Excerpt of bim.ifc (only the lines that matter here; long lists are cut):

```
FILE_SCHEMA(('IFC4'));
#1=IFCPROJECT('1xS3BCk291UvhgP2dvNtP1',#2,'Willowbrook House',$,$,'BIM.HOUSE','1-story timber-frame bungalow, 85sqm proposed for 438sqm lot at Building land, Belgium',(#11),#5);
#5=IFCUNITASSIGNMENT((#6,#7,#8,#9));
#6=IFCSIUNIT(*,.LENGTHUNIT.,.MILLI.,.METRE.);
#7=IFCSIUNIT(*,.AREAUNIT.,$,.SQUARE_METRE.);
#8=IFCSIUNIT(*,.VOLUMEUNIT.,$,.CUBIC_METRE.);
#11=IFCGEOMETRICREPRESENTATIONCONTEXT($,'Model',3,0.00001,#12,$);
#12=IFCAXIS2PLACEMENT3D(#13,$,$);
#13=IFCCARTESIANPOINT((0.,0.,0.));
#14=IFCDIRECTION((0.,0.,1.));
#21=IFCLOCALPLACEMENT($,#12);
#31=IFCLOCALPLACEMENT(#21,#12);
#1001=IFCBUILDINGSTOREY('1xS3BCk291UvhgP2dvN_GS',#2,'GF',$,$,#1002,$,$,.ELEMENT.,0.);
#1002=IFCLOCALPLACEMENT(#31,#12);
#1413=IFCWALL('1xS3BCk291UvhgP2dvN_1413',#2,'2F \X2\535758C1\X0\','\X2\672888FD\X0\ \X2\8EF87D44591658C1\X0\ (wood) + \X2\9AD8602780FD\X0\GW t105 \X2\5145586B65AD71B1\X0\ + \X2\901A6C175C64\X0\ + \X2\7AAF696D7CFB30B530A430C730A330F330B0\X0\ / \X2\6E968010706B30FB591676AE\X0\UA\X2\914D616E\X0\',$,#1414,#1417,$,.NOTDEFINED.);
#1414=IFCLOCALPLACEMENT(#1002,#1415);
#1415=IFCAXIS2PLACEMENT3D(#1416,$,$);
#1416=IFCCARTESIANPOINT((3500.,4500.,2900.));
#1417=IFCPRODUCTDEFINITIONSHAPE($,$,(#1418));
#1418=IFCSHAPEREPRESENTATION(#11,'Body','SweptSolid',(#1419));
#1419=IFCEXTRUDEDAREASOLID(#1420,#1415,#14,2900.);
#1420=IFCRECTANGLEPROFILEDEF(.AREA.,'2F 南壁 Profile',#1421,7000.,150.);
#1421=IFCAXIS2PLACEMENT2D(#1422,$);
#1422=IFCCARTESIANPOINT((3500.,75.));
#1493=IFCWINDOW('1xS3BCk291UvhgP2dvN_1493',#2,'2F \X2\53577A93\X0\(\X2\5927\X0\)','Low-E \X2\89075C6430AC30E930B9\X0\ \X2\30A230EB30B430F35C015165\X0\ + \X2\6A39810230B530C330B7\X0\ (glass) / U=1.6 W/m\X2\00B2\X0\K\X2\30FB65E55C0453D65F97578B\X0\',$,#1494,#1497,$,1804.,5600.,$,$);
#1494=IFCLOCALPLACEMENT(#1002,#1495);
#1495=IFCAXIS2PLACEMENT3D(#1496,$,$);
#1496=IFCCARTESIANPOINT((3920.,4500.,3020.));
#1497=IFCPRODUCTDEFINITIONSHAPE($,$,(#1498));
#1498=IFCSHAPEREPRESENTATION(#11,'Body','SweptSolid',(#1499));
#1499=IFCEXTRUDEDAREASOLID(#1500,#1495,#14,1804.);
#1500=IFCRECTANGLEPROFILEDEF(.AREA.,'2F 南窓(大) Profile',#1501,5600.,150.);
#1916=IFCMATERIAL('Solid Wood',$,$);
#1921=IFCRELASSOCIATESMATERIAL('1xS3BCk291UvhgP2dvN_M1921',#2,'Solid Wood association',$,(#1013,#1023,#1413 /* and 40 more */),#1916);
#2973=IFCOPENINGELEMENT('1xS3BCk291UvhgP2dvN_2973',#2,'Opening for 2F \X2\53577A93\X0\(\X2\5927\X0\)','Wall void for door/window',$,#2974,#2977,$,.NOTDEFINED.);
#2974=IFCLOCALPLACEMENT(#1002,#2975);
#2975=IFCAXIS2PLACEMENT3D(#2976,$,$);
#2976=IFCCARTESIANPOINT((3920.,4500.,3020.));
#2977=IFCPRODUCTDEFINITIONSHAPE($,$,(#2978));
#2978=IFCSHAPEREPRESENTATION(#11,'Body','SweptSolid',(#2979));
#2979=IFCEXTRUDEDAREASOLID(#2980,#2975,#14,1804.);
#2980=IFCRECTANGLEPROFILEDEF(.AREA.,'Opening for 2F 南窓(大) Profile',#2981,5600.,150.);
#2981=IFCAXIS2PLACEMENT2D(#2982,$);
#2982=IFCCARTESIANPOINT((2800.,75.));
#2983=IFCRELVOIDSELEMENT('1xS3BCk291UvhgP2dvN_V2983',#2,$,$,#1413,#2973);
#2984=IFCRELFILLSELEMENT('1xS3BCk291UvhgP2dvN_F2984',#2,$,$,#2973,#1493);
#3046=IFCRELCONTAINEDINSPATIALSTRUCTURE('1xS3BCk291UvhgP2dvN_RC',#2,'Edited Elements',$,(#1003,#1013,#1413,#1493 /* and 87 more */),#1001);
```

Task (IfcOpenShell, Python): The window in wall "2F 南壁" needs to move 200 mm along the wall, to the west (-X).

```python
import ifcopenshell
import ifcopenshell.api.geometry
import ifcopenshell.util.placement

model = ifcopenshell.open("bim.ifc")

window = model.by_guid("1xS3BCk291UvhgP2dvN_1493")
opening = window.FillsVoids[0].RelatingOpeningElement
wall = opening.VoidsElements[0].RelatingBuildingElement

wall_matrix = ifcopenshell.util.placement.get_local_placement(wall.ObjectPlacement)
shift = wall_matrix[:3, 0] * -200.0
before = ifcopenshell.util.placement.get_local_placement(window.ObjectPlacement)[:3, 3].copy()

# The window is not placed relative to its opening, so move both.
for product in (opening, window):
    matrix = ifcopenshell.util.placement.get_local_placement(product.ObjectPlacement)
    matrix[:3, 3] += shift
    ifcopenshell.api.geometry.edit_object_placement(model, product=product, matrix=matrix, is_si=False)

after = ifcopenshell.util.placement.get_local_placement(window.ObjectPlacement)[:3, 3]
print("window moved by", (after - before).round(3) + 0.0)

model.write("bim_edited.ifc")
```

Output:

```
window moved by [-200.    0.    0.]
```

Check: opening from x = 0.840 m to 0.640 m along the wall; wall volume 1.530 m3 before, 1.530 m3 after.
